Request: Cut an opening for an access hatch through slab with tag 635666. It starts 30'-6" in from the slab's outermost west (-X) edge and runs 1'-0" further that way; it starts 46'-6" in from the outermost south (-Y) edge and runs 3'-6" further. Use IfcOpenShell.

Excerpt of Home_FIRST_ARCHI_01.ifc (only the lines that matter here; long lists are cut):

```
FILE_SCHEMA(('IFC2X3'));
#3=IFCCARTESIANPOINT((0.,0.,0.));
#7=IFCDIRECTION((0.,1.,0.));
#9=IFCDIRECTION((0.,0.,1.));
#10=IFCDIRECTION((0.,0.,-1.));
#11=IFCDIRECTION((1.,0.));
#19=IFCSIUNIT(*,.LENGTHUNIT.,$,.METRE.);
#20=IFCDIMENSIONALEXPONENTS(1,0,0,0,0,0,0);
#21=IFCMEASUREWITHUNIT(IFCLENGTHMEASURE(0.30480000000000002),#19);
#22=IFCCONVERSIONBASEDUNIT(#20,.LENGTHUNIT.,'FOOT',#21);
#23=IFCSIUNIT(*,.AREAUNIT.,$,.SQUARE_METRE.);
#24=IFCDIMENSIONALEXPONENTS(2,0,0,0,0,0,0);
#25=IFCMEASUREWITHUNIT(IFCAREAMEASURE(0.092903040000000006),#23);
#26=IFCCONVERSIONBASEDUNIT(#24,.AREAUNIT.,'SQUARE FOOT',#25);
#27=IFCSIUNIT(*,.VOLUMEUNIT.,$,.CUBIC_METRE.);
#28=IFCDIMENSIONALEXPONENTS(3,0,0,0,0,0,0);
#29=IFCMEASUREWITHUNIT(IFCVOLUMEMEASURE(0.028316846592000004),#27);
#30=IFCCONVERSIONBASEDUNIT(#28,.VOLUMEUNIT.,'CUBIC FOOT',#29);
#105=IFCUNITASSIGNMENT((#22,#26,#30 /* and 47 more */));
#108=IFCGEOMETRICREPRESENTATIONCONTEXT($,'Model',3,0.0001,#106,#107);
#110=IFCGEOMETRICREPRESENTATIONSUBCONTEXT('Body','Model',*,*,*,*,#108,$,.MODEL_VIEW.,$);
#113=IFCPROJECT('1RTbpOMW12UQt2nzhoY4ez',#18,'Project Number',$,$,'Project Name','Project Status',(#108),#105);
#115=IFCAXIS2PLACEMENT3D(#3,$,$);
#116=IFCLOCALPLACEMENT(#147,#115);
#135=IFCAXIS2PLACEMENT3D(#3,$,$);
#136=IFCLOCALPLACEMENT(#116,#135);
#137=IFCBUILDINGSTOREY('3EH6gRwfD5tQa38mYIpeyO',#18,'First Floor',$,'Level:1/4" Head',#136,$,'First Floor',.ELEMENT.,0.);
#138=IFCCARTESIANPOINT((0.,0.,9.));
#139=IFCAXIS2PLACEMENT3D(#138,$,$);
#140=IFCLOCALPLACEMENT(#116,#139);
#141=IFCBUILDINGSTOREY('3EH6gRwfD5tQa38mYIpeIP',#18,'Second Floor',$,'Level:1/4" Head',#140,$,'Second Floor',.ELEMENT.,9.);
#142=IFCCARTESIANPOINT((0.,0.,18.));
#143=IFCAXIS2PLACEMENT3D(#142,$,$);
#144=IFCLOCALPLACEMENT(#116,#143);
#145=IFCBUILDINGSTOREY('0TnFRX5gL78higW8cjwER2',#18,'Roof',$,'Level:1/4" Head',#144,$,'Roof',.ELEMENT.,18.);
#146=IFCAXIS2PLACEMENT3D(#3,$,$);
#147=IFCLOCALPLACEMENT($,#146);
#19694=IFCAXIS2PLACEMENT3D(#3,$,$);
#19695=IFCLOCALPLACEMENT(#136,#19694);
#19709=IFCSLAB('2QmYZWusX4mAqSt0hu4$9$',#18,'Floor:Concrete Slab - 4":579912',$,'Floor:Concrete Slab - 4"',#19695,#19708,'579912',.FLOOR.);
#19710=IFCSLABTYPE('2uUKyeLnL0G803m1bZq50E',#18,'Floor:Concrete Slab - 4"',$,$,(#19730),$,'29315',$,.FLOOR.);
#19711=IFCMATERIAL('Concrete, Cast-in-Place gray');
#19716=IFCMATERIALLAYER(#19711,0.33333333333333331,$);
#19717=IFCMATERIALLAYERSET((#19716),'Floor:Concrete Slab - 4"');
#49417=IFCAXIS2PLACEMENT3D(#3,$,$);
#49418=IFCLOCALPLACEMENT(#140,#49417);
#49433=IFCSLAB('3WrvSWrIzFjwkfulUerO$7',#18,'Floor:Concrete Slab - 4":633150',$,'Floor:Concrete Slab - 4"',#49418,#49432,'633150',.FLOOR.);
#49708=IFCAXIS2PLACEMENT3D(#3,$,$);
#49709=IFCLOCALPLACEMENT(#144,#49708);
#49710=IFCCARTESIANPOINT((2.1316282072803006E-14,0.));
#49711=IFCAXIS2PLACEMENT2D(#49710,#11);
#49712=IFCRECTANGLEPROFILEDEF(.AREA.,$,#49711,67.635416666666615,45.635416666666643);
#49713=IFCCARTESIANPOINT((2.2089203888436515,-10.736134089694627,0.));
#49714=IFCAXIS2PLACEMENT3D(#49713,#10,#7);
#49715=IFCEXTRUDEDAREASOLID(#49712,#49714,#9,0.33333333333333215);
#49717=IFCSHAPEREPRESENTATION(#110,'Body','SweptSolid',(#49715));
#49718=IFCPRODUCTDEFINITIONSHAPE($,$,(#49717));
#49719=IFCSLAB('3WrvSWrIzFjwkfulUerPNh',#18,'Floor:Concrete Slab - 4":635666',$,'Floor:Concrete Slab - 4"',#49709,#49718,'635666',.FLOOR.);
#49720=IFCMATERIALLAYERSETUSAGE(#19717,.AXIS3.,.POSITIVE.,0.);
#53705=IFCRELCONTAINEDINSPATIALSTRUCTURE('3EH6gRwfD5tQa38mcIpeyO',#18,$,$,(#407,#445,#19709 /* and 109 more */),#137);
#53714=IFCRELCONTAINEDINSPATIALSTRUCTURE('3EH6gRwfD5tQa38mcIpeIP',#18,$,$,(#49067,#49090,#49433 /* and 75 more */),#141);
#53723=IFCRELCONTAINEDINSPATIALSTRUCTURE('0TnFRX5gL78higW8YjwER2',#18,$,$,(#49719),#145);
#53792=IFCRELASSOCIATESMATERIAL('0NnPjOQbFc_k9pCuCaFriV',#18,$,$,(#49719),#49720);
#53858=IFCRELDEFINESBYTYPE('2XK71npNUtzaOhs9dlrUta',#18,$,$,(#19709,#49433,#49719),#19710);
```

```python
import numpy as np
import ifcopenshell
import ifcopenshell.api.feature
import ifcopenshell.api.geometry
import ifcopenshell.api.root
import ifcopenshell.geom
import ifcopenshell.util.placement
import ifcopenshell.util.representation
import ifcopenshell.util.shape
import ifcopenshell.util.unit

model = ifcopenshell.open("Home_FIRST_ARCHI_01.ifc")
unit_scale = ifcopenshell.util.unit.calculate_unit_scale(model)
settings = ifcopenshell.geom.settings()


def volume(element):
    """Net volume in cubic metres, openings subtracted."""
    shape = ifcopenshell.geom.create_shape(settings, element)
    return ifcopenshell.util.shape.get_volume(shape.geometry)


slab = model.by_guid("3WrvSWrIzFjwkfulUerPNh")
before = volume(slab)

# Extent in the slab's own axes, in metres. The edges named are its -X and -Y sides.
slab_shape = ifcopenshell.geom.create_shape(settings, slab)
vertices = ifcopenshell.util.shape.get_vertices(slab_shape.geometry)
x_min, y_min, bottom = vertices.min(axis=0)
top = vertices[:, 2].max()

opening = ifcopenshell.api.root.create_entity(model, ifc_class="IfcOpeningElement", name="Access hatch opening")
context = ifcopenshell.util.representation.get_context(model, "Model", "Body", "MODEL_VIEW")
width, depth = 0.3048, 1.0668
outline = [(0.0, 0.0), (width, 0.0), (width, depth), (0.0, depth), (0.0, 0.0)]
# Overshoot both faces by 50 mm so the cut is clean.
shape = ifcopenshell.api.geometry.add_slab_representation(
    model, context=context, depth=top - bottom + 0.1, polyline=outline
)
ifcopenshell.api.geometry.assign_representation(model, product=opening, representation=shape)

matrix = ifcopenshell.util.placement.get_local_placement(slab.ObjectPlacement)
matrix[:, 3] = matrix @ np.append(np.array([x_min + 9.2964, y_min + 14.1732, bottom - 0.05]) / unit_scale, 1.0)
ifcopenshell.api.geometry.edit_object_placement(model, product=opening, matrix=matrix, is_si=False)
ifcopenshell.api.feature.add_feature(model, feature=opening, element=slab)

after = volume(slab)

print(f"slab volume {before:.3f} -> {after:.3f} m3")

model.write("Home_FIRST_ARCHI_01_updated.ifc")
```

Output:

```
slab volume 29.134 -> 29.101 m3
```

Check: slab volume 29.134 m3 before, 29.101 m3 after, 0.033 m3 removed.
